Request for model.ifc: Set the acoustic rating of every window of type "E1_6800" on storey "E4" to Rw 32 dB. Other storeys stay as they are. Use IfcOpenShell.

First a look at what the model holds.

```python
import ifcopenshell
import ifcopenshell.util.element

model = ifcopenshell.open("model.ifc")
print(model.schema)
storey = next(s for s in model.by_type("IfcBuildingStorey") if s.Name == "E4")
windows = [e for e in ifcopenshell.util.element.get_decomposition(storey) if e.is_a("IfcWindow")]
seen = {}
for e in windows:
    element_type = ifcopenshell.util.element.get_type(e)
    key = (element_type.Name if element_type != e and element_type else None, ifcopenshell.util.element.get_pset(e, "Pset_WindowCommon", "AcousticRating"))
    seen[key] = seen.get(key, 0) + 1
for (name, value), count in sorted(seen.items(), key=str):
    print(count, "x", name, "|", value)
```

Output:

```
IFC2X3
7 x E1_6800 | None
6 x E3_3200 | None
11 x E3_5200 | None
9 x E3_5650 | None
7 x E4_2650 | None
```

```python
import ifcopenshell
import ifcopenshell.api.pset
import ifcopenshell.util.element

model = ifcopenshell.open("model.ifc")

storey = next(s for s in model.by_type("IfcBuildingStorey") if s.Name == "E4")
windows = [e for e in ifcopenshell.util.element.get_decomposition(storey) if e.is_a("IfcWindow")]

count = 0
for e in windows:
    element_type = ifcopenshell.util.element.get_type(e)
    if element_type in (None, e) or element_type.Name != "E1_6800":
        continue
    # add_pset returns the element's existing set when there is one.
    pset = ifcopenshell.api.pset.add_pset(model, product=e, name="Pset_WindowCommon")
    ifcopenshell.api.pset.edit_pset(model, pset=pset, properties={"AcousticRating": "Rw 32 dB"})
    count += 1

print(count, "windows updated")

model.write("model-out.ifc")
```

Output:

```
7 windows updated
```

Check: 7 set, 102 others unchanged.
